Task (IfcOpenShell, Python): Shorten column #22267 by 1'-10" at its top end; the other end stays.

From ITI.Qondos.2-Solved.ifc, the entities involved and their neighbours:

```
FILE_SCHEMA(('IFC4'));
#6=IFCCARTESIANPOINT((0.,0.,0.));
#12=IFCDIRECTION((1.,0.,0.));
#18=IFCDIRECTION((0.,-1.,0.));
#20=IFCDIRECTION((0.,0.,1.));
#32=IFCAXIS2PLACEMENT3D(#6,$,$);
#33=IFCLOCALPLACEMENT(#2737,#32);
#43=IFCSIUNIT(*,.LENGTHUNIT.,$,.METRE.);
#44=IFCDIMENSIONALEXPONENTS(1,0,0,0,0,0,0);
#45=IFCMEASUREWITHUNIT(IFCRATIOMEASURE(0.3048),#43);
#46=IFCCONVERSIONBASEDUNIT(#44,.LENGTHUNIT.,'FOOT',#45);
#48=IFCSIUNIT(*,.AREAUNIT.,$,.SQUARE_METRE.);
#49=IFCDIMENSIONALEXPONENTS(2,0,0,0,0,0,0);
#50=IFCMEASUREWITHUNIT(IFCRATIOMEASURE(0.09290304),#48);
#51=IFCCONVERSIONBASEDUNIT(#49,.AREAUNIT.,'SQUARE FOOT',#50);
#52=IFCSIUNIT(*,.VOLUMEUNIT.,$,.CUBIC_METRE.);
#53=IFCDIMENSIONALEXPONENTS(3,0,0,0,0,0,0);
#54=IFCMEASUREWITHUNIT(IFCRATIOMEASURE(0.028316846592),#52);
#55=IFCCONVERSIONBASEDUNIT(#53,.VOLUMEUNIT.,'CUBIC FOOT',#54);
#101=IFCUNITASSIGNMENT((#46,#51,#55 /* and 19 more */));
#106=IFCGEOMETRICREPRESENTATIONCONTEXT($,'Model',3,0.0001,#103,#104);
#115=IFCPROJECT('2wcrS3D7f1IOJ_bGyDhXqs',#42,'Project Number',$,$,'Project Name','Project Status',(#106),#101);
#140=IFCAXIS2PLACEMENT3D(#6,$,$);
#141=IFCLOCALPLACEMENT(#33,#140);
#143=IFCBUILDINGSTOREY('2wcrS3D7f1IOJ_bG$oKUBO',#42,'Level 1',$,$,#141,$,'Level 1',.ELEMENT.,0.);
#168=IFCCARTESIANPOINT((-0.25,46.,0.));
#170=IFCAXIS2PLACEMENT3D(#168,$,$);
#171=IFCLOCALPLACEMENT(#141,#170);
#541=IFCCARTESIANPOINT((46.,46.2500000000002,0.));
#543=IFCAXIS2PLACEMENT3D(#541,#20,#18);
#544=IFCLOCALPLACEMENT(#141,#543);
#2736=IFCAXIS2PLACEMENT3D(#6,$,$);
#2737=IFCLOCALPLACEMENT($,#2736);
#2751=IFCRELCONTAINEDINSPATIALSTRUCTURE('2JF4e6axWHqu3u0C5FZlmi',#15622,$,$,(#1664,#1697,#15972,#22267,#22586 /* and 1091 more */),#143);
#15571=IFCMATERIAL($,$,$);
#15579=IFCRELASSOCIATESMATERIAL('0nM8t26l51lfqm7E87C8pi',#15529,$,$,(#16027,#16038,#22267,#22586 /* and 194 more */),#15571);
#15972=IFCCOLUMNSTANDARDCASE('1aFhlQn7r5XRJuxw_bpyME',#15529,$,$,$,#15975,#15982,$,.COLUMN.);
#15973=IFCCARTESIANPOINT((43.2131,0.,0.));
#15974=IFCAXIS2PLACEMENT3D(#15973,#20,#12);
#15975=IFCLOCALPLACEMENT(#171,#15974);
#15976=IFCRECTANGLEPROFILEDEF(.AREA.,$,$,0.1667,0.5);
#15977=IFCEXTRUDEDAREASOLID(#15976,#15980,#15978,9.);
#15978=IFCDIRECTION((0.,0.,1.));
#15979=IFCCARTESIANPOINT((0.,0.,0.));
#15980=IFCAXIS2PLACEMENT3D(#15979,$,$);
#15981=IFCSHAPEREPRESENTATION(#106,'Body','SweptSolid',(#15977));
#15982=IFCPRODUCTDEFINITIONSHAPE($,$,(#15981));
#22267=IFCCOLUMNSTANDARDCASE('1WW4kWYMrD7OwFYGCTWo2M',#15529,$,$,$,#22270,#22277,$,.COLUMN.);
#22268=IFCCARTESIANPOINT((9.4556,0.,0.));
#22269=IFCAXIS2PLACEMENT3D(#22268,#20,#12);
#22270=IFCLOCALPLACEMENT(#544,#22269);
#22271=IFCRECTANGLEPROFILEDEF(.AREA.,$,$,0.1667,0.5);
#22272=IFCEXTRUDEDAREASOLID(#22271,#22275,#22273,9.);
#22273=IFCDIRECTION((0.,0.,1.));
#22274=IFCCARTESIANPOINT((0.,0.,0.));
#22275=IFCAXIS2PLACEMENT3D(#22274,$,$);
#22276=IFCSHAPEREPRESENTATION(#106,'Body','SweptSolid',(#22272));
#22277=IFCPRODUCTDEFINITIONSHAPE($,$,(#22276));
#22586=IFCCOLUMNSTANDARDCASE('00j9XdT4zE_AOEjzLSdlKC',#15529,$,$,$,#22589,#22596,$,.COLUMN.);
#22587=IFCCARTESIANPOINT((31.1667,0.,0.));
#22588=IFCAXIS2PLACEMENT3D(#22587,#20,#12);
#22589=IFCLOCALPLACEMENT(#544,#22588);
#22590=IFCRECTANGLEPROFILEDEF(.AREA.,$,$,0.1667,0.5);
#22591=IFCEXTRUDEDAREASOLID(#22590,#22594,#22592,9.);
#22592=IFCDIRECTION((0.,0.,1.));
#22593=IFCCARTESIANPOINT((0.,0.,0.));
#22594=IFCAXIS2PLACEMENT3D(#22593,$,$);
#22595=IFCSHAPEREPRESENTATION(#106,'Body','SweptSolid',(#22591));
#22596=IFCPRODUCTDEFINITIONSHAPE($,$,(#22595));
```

```python
import ifcopenshell
import ifcopenshell.util.unit

model = ifcopenshell.open("ITI.Qondos.2-Solved.ifc")
unit_scale = ifcopenshell.util.unit.calculate_unit_scale(model)

member = model.by_guid("1WW4kWYMrD7OwFYGCTWo2M")
change = -22 * 0.0254 / unit_scale

# The extrusion runs towards the end named, so only its depth changes.
body = next(r for r in member.Representation.Representations if r.RepresentationIdentifier == "Body")
solid = body.Items[0]
old_length = solid.Depth
solid.Depth += change

print(f"length {old_length:g} -> {solid.Depth:g}")

model.write("ITI.Qondos.2-Solved_updated.ifc")
```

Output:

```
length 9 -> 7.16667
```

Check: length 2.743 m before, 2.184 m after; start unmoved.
